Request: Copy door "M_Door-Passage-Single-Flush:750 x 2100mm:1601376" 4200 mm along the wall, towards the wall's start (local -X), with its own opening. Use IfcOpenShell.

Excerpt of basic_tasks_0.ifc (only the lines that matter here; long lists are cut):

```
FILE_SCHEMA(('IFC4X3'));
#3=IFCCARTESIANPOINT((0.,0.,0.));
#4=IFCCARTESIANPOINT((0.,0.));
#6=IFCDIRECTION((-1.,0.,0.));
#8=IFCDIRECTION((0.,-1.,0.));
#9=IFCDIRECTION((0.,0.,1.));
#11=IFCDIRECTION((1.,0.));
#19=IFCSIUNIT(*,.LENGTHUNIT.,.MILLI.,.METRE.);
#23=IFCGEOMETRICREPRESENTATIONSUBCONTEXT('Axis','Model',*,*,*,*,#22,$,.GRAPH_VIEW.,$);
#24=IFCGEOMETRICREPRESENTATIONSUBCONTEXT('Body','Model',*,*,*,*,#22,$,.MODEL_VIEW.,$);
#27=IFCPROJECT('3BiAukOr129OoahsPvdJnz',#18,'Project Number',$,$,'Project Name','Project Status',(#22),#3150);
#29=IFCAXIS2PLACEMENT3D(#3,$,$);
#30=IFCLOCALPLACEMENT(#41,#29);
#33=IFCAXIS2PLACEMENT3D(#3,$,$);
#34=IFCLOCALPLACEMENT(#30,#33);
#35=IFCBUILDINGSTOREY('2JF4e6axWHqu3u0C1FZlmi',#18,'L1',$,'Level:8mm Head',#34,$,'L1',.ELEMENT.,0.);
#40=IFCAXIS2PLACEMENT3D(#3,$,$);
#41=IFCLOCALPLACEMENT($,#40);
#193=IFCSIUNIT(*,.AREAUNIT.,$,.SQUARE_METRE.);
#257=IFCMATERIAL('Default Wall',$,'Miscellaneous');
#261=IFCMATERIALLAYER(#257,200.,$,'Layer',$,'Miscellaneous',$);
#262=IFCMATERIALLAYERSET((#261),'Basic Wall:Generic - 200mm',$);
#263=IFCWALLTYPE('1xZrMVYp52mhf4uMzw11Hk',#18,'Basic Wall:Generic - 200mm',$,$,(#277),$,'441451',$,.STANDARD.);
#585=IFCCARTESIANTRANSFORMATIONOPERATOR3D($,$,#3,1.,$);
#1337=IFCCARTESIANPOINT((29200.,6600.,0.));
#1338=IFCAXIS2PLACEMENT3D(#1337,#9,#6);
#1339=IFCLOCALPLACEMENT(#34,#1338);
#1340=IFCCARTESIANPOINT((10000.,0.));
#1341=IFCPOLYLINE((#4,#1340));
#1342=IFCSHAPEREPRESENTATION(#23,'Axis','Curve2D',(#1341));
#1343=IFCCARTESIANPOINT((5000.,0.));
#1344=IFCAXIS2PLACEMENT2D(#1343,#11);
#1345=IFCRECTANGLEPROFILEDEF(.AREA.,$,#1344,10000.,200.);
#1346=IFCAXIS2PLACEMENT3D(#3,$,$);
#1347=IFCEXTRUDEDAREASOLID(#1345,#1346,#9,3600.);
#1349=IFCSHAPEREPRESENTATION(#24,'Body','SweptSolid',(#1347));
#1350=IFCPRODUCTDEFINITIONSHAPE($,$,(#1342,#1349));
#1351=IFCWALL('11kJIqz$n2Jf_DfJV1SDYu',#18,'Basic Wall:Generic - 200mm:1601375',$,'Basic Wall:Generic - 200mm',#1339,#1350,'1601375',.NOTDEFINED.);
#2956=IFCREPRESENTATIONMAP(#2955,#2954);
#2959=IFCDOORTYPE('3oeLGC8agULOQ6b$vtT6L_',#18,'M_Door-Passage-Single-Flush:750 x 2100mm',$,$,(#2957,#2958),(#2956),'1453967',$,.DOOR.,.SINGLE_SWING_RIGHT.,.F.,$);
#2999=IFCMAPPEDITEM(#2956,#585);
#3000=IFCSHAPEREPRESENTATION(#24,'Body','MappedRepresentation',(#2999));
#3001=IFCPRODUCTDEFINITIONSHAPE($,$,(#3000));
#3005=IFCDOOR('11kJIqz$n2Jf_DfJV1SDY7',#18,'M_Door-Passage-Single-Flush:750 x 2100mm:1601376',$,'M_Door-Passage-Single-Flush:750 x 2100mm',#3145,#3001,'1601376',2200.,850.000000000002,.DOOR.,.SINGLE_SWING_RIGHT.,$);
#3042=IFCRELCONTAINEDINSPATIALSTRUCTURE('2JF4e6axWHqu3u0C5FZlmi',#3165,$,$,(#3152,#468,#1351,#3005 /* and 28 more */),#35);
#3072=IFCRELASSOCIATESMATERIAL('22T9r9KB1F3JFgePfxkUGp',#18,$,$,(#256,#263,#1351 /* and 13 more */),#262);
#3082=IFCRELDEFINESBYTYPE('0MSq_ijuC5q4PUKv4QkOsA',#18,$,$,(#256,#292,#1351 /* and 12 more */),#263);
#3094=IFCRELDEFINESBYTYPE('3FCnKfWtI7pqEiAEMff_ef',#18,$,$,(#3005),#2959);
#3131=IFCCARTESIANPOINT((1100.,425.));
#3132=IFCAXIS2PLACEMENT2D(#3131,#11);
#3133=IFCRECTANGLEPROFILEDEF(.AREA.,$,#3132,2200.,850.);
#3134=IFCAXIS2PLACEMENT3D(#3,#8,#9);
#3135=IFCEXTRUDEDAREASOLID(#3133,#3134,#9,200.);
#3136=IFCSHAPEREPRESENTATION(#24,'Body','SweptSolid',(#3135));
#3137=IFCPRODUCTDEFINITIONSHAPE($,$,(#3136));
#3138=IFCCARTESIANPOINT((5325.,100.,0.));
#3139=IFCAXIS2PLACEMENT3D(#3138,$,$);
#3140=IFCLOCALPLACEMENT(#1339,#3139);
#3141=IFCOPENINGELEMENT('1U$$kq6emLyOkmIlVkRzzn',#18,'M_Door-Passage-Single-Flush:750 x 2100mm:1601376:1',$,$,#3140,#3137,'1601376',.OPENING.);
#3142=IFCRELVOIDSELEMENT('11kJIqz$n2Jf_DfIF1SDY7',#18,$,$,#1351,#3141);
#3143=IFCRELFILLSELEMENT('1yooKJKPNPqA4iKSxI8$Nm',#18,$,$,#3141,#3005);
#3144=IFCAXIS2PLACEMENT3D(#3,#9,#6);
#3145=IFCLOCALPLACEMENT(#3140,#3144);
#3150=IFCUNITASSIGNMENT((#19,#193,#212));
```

```python
import ifcopenshell
import ifcopenshell.api.feature
import ifcopenshell.api.geometry
import ifcopenshell.api.root
import ifcopenshell.geom
import ifcopenshell.util.element
import ifcopenshell.util.placement
import ifcopenshell.util.shape

model = ifcopenshell.open("basic_tasks_0.ifc")
settings = ifcopenshell.geom.settings()


def volume(element):
    """Net volume in cubic metres, openings subtracted."""
    shape = ifcopenshell.geom.create_shape(settings, element)
    return ifcopenshell.util.shape.get_volume(shape.geometry)


def reuse_history(source, copy):
    """copy_class also copies each property set's owner history, people and application; keep the originals."""
    for rel in copy.IsDefinedBy:
        if rel.is_a("IfcRelDefinesByProperties") and (history := rel.RelatingPropertyDefinition.OwnerHistory):
            rel.RelatingPropertyDefinition.OwnerHistory = source.OwnerHistory
            ifcopenshell.util.element.remove_deep2(model, history)


door = model.by_guid("11kJIqz$n2Jf_DfJV1SDY7")
opening = door.FillsVoids[0].RelatingOpeningElement
wall = opening.VoidsElements[0].RelatingBuildingElement
before = volume(wall)
shift = ifcopenshell.util.placement.get_local_placement(wall.ObjectPlacement)[:3, 0] * -4200.0

# copy_class copies the void relationship, type, container and properties, but no geometry.
new_opening = ifcopenshell.api.root.copy_class(model, product=opening)
new_opening.Representation = ifcopenshell.util.element.copy_deep(
    model, opening.Representation, exclude=["IfcGeometricRepresentationContext", "IfcRepresentationMap"]
)
new_opening.Name = "M_Door-Passage-Single-Flush:750 x 2100mm"
new_opening.Tag = None
new_door = ifcopenshell.api.root.copy_class(model, product=door)
new_door.Representation = ifcopenshell.util.element.copy_deep(
    model, door.Representation, exclude=["IfcGeometricRepresentationContext", "IfcRepresentationMap"]
)
new_door.Name = "M_Door-Passage-Single-Flush:750 x 2100mm"
new_door.Tag = None
reuse_history(door, new_door)
ifcopenshell.api.feature.add_filling(model, opening=new_opening, element=new_door)

for old, new in ((opening, new_opening), (door, new_door)):
    matrix = ifcopenshell.util.placement.get_local_placement(old.ObjectPlacement)
    matrix[:3, 3] += shift
    ifcopenshell.api.geometry.edit_object_placement(model, product=new, matrix=matrix, is_si=False)

after = volume(wall)

print(f"wall volume {before:.3f} -> {after:.3f} m3")

model.write("basic_tasks_0_rev.ifc")
```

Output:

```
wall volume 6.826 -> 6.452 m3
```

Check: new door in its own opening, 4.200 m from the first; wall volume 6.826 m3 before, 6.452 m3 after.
